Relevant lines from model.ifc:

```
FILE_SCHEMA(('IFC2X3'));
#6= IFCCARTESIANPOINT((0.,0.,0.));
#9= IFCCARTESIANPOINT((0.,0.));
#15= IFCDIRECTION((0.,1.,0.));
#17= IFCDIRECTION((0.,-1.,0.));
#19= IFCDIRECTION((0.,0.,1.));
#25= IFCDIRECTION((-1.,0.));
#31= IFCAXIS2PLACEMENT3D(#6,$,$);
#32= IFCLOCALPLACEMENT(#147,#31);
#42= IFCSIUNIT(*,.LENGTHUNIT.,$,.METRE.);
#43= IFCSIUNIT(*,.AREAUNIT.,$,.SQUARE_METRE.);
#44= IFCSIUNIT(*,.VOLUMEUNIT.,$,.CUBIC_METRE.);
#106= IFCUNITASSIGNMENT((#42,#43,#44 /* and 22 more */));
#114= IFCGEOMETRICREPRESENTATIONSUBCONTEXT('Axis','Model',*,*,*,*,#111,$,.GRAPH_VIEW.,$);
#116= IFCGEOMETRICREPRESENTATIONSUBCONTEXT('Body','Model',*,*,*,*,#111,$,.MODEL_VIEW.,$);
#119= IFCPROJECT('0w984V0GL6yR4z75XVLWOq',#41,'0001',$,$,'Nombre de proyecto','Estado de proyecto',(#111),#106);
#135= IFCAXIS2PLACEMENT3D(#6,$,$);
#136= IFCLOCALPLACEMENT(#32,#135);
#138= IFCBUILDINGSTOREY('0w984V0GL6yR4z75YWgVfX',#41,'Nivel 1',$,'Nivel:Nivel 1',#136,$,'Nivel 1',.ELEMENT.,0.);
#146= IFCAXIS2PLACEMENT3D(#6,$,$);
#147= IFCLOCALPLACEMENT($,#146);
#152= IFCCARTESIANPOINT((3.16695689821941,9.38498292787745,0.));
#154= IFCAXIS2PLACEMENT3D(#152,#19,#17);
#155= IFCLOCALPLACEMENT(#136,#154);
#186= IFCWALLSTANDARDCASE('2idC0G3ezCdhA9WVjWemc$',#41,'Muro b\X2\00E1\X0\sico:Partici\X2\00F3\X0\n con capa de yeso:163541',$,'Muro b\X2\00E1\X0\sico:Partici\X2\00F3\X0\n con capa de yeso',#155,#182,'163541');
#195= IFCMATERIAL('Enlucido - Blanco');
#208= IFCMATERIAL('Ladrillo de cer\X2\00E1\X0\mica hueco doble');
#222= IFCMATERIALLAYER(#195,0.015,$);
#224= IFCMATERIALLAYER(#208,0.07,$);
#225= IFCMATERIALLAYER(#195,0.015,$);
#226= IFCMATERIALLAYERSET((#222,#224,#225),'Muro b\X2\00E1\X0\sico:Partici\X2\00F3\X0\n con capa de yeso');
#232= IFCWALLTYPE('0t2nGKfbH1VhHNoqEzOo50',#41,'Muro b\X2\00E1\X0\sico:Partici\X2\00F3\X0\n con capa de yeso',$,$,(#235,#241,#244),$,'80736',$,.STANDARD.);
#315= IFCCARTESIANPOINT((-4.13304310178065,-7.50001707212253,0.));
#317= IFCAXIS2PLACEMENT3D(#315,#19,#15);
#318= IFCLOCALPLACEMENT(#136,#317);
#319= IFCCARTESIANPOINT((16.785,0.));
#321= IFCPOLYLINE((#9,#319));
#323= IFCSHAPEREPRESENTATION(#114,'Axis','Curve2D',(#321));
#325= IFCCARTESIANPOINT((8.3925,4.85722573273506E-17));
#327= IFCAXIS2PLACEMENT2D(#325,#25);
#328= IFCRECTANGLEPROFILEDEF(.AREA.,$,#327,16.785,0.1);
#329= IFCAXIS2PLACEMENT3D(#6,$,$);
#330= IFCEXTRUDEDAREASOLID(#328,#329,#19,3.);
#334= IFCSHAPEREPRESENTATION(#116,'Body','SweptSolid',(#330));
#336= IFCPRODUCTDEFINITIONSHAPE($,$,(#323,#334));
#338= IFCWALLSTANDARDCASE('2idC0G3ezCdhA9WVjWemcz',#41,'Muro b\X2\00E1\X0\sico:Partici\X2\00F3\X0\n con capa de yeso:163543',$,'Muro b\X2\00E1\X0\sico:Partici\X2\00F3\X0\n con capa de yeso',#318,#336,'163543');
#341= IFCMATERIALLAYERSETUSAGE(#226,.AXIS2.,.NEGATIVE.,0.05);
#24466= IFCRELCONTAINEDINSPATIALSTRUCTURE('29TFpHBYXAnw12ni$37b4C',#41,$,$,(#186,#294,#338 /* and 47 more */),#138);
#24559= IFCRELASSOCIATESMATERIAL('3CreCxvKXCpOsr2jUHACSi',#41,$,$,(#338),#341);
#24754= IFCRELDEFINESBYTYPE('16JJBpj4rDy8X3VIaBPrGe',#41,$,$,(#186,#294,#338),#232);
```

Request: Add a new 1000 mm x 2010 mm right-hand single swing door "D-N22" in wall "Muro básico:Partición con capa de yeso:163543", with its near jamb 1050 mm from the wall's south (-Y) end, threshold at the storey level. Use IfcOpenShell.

```python
import numpy as np
import ifcopenshell
import ifcopenshell.api.feature
import ifcopenshell.api.geometry
import ifcopenshell.api.root
import ifcopenshell.api.spatial
import ifcopenshell.api.type
import ifcopenshell.geom
import ifcopenshell.util.element
import ifcopenshell.util.placement
import ifcopenshell.util.representation
import ifcopenshell.util.shape
import ifcopenshell.util.unit

model = ifcopenshell.open("model.ifc")
unit_scale = ifcopenshell.util.unit.calculate_unit_scale(model)
settings = ifcopenshell.geom.settings()


def volume(element):
    """Net volume in cubic metres, openings subtracted."""
    shape = ifcopenshell.geom.create_shape(settings, element)
    return ifcopenshell.util.shape.get_volume(shape.geometry)


wall = model.by_guid("2idC0G3ezCdhA9WVjWemcz")
storey = ifcopenshell.util.element.get_container(wall, ifc_class="IfcBuildingStorey")
context = ifcopenshell.util.representation.get_context(model, "Model", "Body", "MODEL_VIEW")
before = volume(wall)

width, height, from_end, sill = 1, 2.01, 1.05, 0.0  # metres

# The wall runs along its own X axis, and the end named is its -X end.
wall_shape = ifcopenshell.geom.create_shape(settings, wall)
x, y, z = ifcopenshell.util.shape.get_vertices(wall_shape.geometry).T
start = x.min() + from_end
face, thickness = float(y.min()), float(y.max() - y.min())
wall_matrix = ifcopenshell.util.placement.get_local_placement(wall.ObjectPlacement)
level = ifcopenshell.util.placement.get_local_placement(storey.ObjectPlacement)[2, 3]


def in_wall(x, y):
    """Placement at x, y metres in the wall's axes, at sill height."""
    matrix = wall_matrix.copy()
    matrix[:, 3] = wall_matrix @ np.array([x / unit_scale, y / unit_scale, 0.0, 1.0])
    matrix[2, 3] = level + sill / unit_scale
    return matrix


# Opening: a box that overshoots both wall faces by 50 mm.
opening = ifcopenshell.api.root.create_entity(model, ifc_class="IfcOpeningElement")
box = ifcopenshell.api.geometry.add_wall_representation(
    model, context=context, length=width, height=height, thickness=thickness + 0.1
)
ifcopenshell.api.geometry.assign_representation(model, product=opening, representation=box)
ifcopenshell.api.geometry.edit_object_placement(model, product=opening, matrix=in_wall(start, face - 0.05), is_si=False)
ifcopenshell.api.feature.add_feature(model, feature=opening, element=wall)

door = ifcopenshell.api.root.create_entity(model, ifc_class="IfcDoor", name="D-N22")
door.OverallWidth, door.OverallHeight = width / unit_scale, height / unit_scale
body = ifcopenshell.api.geometry.add_door_representation(
    model,
    context=context,
    overall_width=door.OverallWidth,
    overall_height=door.OverallHeight,
    operation_type="SINGLE_SWING_RIGHT",
    lining_properties={"LiningDepth": thickness / unit_scale, "ThresholdDepth": thickness / unit_scale},
)
ifcopenshell.api.geometry.assign_representation(model, product=door, representation=body)
ifcopenshell.api.spatial.assign_container(model, products=[door], relating_structure=storey)
fills = ifcopenshell.api.feature.add_filling(model, opening=opening, element=door)
fills.OwnerHistory = door.OwnerHistory  # required in IFC2X3

# IFC2X3 keeps the operation on the door style.
style = ifcopenshell.api.root.create_entity(model, ifc_class="IfcDoorStyle", name="D-N22")
style.OperationType, style.ConstructionType = "SINGLE_SWING_RIGHT", "NOTDEFINED"
style.ParameterTakesPrecedence = style.Sizeable = False
ifcopenshell.api.type.assign_type(model, related_objects=[door], relating_type=style)

# The lining spans the wall, so the door starts at the wall face.
ifcopenshell.api.geometry.edit_object_placement(model, product=door, matrix=in_wall(start, face), is_si=False)

after = volume(wall)

print(f"wall volume {before:.3f} -> {after:.3f} m3")

model.write("model_rev.ifc")
```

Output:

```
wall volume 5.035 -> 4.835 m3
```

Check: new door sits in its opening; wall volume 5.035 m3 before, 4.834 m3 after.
